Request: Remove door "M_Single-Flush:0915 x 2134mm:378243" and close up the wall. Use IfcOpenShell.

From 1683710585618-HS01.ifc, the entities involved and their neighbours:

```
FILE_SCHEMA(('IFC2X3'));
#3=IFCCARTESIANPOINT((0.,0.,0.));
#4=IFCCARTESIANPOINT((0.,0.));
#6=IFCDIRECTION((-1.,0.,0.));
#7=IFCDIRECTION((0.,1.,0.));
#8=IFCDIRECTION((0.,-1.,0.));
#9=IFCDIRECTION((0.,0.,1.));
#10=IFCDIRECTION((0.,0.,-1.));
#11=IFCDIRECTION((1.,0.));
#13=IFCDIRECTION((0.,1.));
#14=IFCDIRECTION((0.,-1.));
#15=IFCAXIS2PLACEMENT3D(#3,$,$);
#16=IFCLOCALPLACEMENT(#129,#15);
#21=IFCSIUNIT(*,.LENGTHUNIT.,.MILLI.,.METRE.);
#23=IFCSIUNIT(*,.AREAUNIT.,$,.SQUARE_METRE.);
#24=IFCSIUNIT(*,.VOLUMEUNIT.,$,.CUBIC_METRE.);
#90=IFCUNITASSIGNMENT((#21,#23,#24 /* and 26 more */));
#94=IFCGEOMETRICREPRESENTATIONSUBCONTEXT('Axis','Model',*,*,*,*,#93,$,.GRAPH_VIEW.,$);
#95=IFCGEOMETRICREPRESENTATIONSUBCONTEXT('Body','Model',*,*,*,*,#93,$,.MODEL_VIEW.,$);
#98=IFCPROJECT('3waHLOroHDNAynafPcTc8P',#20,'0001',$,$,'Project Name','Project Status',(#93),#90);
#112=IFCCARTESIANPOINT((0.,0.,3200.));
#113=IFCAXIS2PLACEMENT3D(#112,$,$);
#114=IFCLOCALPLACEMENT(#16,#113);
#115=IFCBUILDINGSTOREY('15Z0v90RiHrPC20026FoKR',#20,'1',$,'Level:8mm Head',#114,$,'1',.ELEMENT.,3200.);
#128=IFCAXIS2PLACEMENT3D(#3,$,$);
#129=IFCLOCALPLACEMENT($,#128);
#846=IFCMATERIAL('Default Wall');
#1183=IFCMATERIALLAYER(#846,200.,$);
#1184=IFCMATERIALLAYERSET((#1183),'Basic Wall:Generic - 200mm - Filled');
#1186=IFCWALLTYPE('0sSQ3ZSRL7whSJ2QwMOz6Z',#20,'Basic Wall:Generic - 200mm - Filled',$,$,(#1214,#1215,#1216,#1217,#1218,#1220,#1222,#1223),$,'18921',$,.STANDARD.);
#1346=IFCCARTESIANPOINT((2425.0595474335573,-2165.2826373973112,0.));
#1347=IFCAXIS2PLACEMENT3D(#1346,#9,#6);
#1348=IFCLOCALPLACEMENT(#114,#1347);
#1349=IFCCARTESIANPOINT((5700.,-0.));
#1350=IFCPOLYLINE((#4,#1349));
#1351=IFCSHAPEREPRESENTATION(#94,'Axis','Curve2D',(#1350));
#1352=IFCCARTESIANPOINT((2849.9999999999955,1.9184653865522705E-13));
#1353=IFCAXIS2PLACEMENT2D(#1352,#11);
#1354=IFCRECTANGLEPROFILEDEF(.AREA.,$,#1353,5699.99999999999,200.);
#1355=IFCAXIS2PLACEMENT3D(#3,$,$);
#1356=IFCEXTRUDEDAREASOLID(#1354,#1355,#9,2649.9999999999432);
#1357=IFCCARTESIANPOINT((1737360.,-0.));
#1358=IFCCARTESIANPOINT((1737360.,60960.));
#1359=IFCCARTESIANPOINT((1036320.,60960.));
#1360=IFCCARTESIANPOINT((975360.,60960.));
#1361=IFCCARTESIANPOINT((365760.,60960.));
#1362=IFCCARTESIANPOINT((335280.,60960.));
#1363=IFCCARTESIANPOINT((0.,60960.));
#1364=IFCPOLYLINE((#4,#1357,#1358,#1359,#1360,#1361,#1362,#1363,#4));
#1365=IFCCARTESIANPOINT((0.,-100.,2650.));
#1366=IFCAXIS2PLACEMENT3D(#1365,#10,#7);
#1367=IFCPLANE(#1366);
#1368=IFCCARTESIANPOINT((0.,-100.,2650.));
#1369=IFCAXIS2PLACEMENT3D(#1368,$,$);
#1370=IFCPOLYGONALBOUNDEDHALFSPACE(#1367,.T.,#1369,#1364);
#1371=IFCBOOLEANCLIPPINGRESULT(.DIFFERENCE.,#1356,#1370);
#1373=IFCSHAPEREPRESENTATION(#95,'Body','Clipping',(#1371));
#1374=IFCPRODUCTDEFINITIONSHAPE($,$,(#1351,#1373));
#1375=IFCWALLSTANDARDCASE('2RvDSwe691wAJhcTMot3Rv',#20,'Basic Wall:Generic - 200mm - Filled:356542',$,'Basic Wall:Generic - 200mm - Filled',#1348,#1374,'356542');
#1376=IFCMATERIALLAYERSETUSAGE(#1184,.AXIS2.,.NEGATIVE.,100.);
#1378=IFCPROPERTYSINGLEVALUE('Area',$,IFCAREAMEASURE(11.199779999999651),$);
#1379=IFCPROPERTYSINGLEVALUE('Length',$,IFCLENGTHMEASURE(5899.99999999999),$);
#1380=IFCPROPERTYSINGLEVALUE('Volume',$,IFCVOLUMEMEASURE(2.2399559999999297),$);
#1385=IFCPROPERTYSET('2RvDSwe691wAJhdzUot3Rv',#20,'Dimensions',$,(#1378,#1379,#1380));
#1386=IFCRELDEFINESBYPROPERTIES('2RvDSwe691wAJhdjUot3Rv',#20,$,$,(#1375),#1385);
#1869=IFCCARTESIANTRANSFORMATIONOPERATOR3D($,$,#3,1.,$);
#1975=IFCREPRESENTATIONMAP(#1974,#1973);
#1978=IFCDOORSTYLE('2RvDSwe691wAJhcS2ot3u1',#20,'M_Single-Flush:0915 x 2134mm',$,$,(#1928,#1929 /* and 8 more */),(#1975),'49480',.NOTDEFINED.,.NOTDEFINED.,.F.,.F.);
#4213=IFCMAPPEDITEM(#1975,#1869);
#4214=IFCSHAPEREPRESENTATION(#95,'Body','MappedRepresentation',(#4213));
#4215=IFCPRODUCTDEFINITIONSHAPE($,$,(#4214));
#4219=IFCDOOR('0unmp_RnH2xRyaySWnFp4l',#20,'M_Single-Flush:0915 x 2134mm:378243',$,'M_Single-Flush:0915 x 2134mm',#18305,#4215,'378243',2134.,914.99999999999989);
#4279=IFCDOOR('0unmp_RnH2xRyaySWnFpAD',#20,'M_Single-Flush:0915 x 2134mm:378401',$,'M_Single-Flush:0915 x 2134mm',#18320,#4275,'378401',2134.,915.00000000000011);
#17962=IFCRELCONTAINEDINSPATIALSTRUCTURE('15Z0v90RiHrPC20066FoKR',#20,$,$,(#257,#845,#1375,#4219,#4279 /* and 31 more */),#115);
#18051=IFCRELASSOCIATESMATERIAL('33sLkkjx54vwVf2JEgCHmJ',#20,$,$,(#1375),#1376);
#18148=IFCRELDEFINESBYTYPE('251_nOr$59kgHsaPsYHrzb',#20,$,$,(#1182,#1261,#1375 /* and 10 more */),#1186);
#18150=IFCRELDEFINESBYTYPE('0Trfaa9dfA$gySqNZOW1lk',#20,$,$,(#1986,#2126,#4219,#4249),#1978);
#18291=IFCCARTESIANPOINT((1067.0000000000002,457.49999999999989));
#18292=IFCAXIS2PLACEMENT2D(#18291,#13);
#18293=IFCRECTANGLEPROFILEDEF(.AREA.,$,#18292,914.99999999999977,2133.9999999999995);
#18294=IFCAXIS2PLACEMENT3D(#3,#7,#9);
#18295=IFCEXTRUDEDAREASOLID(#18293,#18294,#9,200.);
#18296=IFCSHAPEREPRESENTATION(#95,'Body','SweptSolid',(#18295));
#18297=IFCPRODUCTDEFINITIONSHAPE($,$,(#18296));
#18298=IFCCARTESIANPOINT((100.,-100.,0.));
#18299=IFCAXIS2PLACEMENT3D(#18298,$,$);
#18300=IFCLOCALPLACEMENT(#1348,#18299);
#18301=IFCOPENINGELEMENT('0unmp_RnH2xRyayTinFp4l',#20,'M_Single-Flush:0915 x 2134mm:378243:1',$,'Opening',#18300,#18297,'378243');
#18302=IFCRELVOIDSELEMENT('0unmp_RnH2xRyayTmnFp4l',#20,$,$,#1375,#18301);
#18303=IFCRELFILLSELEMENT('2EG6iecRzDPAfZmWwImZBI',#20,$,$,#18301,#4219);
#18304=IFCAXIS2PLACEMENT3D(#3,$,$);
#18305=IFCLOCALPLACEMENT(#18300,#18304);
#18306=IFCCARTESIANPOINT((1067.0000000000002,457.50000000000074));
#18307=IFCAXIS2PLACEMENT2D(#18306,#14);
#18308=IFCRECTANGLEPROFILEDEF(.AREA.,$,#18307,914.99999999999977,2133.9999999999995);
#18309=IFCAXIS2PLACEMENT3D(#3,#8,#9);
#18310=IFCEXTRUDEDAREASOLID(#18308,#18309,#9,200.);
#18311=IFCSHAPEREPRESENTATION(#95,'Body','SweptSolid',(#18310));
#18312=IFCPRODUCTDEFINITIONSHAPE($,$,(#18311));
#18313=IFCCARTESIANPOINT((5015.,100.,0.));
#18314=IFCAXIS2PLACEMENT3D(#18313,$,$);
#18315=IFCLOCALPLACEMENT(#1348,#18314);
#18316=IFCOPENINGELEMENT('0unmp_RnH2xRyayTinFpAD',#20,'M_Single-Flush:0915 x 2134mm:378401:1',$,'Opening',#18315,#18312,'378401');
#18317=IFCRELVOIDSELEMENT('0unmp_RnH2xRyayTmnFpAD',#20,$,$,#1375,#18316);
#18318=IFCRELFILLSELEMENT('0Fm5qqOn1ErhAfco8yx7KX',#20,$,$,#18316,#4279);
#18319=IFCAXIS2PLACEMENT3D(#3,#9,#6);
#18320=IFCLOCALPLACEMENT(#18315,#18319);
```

```python
import ifcopenshell
import ifcopenshell.api.feature
import ifcopenshell.api.pset
import ifcopenshell.api.root
import ifcopenshell.geom
import ifcopenshell.util.element
import ifcopenshell.util.shape
import ifcopenshell.util.unit

model = ifcopenshell.open("1683710585618-HS01.ifc")
area_scale = ifcopenshell.util.unit.calculate_unit_scale(model, "AREAUNIT")
volume_scale = ifcopenshell.util.unit.calculate_unit_scale(model, "VOLUMEUNIT")
settings = ifcopenshell.geom.settings()


def volume(element):
    """Net volume in cubic metres, openings subtracted."""
    shape = ifcopenshell.geom.create_shape(settings, element)
    return ifcopenshell.util.shape.get_volume(shape.geometry)


door = model.by_id(4219)
opening = door.FillsVoids[0].RelatingOpeningElement
wall = opening.VoidsElements[0].RelatingBuildingElement
before = volume(wall)

ifcopenshell.api.root.remove_product(model, product=door)
ifcopenshell.api.feature.remove_feature(model, feature=opening)

after = volume(wall)
thickness = 0.2  # wall thickness in metres

# Update the wall's stored quantities.
pset = model.by_id(ifcopenshell.util.element.get_pset(wall, "Dimensions", should_inherit=False)["id"])
ifcopenshell.api.pset.edit_pset(model, pset=pset, properties={
    "Area": model.create_entity("IfcAreaMeasure", after / thickness / area_scale),
    "Volume": model.create_entity("IfcVolumeMeasure", after / volume_scale),
})

print(f"wall volume {before:.3f} -> {after:.3f} m3")

model.write("1683710585618-HS01_v2.ifc")
```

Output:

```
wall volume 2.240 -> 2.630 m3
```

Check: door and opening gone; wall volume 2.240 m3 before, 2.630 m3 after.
